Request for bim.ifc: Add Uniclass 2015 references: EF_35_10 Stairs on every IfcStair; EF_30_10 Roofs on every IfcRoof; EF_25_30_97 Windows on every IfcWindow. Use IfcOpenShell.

First a look at what the model holds.

```python
import ifcopenshell

model = ifcopenshell.open("bim.ifc")
print(model.schema)
print("classifications:", [c.Name for c in model.by_type("IfcClassification")])
for ifc_class in ("IfcDoor", "IfcRoof", "IfcStair", "IfcWall", "IfcWindow"):
    print(ifc_class, len(model.by_type(ifc_class)))
```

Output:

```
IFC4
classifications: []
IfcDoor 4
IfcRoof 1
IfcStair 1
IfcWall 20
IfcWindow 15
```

```python
import ifcopenshell
import ifcopenshell.api.classification

model = ifcopenshell.open("bim.ifc")

system = ifcopenshell.api.classification.add_classification(model, classification="Uniclass 2015")

codes = {
    "IfcStair": ("EF_35_10", "Stairs"),
    "IfcRoof": ("EF_30_10", "Roofs"),
    "IfcWindow": ("EF_25_30_97", "Windows"),
}
for ifc_class, (code, name) in codes.items():
    products = model.by_type(ifc_class)
    ifcopenshell.api.classification.add_reference(
        model, products=products, classification=system, identification=code, name=name
    )
    print(code, len(products))

model.write("bim_v2.ifc")
```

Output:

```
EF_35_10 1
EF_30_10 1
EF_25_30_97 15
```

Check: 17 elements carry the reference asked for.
